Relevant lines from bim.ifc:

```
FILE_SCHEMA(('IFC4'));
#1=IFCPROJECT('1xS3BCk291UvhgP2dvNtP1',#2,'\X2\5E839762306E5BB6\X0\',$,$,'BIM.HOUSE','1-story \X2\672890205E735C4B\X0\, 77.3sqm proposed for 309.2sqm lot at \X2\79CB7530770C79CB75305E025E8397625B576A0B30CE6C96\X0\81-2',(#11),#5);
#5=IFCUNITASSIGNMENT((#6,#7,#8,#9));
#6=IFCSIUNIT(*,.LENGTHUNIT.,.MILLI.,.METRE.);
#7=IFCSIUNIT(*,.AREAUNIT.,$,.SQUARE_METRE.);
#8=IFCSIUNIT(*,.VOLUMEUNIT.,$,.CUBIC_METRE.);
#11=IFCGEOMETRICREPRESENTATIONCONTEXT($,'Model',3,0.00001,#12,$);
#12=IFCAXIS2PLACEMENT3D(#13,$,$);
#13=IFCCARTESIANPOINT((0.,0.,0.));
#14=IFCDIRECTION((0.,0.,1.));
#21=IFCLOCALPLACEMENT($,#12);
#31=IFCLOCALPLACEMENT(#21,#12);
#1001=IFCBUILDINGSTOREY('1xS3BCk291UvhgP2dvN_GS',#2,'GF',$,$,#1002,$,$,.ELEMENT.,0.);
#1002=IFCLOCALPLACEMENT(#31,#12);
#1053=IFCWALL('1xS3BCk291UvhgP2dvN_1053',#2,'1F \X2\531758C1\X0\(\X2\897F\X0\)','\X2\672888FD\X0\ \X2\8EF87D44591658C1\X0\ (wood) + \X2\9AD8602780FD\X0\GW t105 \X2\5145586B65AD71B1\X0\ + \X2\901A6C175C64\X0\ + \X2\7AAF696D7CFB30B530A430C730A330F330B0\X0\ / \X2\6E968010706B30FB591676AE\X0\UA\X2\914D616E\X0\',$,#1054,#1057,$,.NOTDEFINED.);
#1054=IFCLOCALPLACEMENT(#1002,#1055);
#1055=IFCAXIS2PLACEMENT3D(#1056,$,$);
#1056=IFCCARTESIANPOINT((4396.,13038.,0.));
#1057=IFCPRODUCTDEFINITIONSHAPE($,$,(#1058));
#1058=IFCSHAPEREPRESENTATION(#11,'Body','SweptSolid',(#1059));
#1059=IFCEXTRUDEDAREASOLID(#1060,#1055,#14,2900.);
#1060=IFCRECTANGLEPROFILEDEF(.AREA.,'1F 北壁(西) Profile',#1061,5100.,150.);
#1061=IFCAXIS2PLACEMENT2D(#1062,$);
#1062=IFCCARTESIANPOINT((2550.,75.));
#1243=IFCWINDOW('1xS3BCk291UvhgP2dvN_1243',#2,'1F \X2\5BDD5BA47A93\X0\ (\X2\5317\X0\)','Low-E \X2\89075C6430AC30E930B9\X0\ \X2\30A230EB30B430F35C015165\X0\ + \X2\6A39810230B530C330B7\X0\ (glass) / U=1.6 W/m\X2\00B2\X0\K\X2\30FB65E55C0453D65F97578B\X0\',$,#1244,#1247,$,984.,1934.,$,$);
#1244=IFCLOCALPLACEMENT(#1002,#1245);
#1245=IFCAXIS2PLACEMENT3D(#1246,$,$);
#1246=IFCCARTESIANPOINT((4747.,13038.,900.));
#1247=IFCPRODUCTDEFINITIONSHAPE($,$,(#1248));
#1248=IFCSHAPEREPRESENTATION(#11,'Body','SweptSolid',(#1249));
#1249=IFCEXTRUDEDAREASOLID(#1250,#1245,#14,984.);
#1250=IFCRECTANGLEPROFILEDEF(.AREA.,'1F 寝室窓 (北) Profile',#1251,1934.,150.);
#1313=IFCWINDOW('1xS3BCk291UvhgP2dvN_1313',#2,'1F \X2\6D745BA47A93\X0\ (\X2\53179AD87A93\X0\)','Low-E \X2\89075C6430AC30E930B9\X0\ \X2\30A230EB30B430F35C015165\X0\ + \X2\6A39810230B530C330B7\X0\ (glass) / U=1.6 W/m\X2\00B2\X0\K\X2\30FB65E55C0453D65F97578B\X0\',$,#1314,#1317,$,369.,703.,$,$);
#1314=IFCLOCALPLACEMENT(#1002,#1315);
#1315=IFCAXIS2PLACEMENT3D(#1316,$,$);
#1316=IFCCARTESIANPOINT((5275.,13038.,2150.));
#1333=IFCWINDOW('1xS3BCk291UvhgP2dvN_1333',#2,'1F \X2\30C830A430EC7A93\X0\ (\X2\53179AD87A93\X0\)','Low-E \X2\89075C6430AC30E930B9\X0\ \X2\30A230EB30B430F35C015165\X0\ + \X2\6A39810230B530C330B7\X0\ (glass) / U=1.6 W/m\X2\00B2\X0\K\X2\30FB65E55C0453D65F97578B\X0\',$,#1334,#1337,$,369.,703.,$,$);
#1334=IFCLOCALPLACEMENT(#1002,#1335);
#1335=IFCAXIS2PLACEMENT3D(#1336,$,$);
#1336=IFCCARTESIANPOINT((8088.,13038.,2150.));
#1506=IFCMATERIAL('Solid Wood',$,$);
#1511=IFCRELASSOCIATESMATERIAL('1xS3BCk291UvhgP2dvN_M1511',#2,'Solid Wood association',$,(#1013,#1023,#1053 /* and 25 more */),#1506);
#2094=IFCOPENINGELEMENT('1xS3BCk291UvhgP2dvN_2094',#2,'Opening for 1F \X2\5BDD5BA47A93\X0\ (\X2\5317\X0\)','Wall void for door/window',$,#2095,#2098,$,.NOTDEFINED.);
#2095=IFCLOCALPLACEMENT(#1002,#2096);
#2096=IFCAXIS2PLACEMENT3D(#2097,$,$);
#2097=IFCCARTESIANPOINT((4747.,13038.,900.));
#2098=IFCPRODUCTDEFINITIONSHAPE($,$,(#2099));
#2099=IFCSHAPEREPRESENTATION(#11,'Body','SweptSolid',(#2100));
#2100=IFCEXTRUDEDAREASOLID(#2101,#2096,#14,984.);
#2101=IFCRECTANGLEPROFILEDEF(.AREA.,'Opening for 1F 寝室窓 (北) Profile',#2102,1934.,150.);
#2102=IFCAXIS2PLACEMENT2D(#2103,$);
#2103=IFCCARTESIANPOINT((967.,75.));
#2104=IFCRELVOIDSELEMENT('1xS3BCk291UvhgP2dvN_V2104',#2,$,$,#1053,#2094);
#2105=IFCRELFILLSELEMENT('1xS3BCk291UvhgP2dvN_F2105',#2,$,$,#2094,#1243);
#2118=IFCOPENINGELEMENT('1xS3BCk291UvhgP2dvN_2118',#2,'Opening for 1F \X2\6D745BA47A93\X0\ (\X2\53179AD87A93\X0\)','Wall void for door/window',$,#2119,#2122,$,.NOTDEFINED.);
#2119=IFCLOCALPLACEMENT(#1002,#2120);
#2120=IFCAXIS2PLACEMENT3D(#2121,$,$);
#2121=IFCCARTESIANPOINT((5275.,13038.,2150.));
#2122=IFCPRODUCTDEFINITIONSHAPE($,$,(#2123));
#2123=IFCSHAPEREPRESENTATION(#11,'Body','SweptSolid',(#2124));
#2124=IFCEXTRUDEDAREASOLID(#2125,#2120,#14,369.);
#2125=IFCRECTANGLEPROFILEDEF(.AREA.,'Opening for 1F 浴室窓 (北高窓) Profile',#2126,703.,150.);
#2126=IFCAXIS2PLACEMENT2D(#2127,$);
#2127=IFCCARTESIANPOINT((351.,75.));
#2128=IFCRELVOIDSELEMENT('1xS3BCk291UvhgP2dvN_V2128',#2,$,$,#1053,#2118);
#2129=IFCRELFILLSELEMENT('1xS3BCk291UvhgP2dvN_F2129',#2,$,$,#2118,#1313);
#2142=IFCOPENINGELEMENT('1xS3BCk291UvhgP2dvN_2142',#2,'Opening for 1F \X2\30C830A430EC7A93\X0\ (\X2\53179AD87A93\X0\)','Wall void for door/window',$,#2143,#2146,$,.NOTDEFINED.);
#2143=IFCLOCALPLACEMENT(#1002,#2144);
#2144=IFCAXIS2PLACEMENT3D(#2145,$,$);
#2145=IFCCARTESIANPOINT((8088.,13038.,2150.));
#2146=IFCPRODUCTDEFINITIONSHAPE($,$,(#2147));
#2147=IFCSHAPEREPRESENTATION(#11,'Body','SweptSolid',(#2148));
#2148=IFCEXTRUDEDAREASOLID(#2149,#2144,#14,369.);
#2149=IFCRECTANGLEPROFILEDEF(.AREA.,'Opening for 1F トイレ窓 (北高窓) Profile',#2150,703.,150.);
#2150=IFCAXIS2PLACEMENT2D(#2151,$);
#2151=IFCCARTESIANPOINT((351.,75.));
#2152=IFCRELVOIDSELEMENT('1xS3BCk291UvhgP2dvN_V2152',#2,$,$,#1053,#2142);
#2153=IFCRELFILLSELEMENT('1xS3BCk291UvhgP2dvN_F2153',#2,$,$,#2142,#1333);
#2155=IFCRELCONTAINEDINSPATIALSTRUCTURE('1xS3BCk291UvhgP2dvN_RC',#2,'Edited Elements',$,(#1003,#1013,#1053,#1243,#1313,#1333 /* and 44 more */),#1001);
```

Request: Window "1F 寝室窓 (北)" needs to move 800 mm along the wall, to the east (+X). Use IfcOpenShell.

```python
import ifcopenshell
import ifcopenshell.api.geometry
import ifcopenshell.util.placement
import ifcopenshell.util.unit

model = ifcopenshell.open("bim.ifc")
unit_scale = ifcopenshell.util.unit.calculate_unit_scale(model)

window = model.by_guid("1xS3BCk291UvhgP2dvN_1243")
opening = window.FillsVoids[0].RelatingOpeningElement
wall = opening.VoidsElements[0].RelatingBuildingElement

wall_matrix = ifcopenshell.util.placement.get_local_placement(wall.ObjectPlacement)
shift = wall_matrix[:3, 0] * 0.8 / unit_scale
before = ifcopenshell.util.placement.get_local_placement(window.ObjectPlacement)[:3, 3].copy()

# The window is not placed relative to its opening, so move both.
for product in (opening, window):
    matrix = ifcopenshell.util.placement.get_local_placement(product.ObjectPlacement)
    matrix[:3, 3] += shift
    ifcopenshell.api.geometry.edit_object_placement(model, product=product, matrix=matrix, is_si=False)

after = ifcopenshell.util.placement.get_local_placement(window.ObjectPlacement)[:3, 3]
print("window moved by", (after - before).round(3) + 0.0)

model.write("bim_rev.ifc")
```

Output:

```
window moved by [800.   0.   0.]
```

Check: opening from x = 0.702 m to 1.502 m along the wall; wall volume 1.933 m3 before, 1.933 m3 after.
